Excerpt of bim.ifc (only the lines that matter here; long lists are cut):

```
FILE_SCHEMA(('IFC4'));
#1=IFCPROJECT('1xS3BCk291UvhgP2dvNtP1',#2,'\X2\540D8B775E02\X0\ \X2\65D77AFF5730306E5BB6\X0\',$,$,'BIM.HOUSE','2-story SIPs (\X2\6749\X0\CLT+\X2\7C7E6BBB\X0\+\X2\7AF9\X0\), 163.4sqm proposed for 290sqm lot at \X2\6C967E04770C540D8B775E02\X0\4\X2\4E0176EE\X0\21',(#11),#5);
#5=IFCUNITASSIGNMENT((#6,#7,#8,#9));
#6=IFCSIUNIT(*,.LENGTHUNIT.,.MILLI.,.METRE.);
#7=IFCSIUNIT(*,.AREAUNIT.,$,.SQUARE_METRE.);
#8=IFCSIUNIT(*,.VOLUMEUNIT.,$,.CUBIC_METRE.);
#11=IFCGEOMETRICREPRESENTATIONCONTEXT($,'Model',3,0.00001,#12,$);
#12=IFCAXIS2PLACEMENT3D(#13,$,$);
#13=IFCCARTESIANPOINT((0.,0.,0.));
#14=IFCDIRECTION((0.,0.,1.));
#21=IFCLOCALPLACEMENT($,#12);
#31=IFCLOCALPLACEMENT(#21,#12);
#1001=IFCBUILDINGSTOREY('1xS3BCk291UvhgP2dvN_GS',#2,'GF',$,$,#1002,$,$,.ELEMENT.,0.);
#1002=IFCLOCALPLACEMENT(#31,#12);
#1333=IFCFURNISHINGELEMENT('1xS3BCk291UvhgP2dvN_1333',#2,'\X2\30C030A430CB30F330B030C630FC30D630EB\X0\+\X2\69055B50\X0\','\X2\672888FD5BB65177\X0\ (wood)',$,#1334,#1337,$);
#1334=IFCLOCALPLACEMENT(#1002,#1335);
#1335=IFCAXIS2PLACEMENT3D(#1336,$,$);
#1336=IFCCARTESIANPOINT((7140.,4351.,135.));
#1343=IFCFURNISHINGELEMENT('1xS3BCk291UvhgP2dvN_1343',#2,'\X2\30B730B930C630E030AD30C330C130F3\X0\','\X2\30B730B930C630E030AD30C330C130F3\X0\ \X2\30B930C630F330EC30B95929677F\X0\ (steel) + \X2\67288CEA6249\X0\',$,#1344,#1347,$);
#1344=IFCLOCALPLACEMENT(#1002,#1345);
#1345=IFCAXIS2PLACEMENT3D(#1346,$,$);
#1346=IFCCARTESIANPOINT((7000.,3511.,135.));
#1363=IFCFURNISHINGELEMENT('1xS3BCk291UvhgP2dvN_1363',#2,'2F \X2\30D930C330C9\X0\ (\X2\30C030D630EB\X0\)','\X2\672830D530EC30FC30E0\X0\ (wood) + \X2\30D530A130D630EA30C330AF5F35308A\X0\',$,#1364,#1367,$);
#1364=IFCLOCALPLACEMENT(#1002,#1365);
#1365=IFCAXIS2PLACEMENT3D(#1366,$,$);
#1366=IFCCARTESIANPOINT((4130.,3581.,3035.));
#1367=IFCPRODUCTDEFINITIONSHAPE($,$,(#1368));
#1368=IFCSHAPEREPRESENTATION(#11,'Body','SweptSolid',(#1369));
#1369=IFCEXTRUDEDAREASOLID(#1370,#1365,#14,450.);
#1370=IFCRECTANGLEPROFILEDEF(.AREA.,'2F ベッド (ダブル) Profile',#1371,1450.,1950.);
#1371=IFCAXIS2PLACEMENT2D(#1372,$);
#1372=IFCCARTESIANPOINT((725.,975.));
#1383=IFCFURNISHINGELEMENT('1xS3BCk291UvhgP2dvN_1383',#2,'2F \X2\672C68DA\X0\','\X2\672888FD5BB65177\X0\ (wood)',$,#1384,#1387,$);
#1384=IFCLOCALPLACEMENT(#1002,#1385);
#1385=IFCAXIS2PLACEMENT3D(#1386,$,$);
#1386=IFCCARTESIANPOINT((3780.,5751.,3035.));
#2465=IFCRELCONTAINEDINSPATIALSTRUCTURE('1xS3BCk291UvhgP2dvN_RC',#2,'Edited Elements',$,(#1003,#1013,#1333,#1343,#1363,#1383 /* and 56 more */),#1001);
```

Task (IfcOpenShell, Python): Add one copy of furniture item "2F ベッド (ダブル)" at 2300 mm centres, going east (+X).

```python
import numpy as np
import ifcopenshell
import ifcopenshell.api.geometry
import ifcopenshell.api.root
import ifcopenshell.util.element
import ifcopenshell.util.placement

model = ifcopenshell.open("bim.ifc")


def reuse_history(source, copy):
    """copy_class also copies each property set's owner history, people and application; keep the originals."""
    for rel in copy.IsDefinedBy:
        if rel.is_a("IfcRelDefinesByProperties") and (history := rel.RelatingPropertyDefinition.OwnerHistory):
            rel.RelatingPropertyDefinition.OwnerHistory = source.OwnerHistory
            ifcopenshell.util.element.remove_deep2(model, history)


source = model.by_id(1363)
base = ifcopenshell.util.placement.get_local_placement(source.ObjectPlacement)
step = np.array([1.0, 0.0, 0.0]) * 2300.0

for i in range(1, 2):
    copy = ifcopenshell.api.root.copy_class(model, product=source)
    copy.Representation = ifcopenshell.util.element.copy_deep(
        model, source.Representation, exclude=["IfcGeometricRepresentationContext", "IfcRepresentationMap"]
    )
    reuse_history(source, copy)
    matrix = base.copy()
    matrix[:3, 3] += i * step
    print("added at", matrix[:3, 3].round(3) + 0.0)
    ifcopenshell.api.geometry.edit_object_placement(model, product=copy, matrix=matrix, is_si=False)

model.write("bim_rev.ifc")
```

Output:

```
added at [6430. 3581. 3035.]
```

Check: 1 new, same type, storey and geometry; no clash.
